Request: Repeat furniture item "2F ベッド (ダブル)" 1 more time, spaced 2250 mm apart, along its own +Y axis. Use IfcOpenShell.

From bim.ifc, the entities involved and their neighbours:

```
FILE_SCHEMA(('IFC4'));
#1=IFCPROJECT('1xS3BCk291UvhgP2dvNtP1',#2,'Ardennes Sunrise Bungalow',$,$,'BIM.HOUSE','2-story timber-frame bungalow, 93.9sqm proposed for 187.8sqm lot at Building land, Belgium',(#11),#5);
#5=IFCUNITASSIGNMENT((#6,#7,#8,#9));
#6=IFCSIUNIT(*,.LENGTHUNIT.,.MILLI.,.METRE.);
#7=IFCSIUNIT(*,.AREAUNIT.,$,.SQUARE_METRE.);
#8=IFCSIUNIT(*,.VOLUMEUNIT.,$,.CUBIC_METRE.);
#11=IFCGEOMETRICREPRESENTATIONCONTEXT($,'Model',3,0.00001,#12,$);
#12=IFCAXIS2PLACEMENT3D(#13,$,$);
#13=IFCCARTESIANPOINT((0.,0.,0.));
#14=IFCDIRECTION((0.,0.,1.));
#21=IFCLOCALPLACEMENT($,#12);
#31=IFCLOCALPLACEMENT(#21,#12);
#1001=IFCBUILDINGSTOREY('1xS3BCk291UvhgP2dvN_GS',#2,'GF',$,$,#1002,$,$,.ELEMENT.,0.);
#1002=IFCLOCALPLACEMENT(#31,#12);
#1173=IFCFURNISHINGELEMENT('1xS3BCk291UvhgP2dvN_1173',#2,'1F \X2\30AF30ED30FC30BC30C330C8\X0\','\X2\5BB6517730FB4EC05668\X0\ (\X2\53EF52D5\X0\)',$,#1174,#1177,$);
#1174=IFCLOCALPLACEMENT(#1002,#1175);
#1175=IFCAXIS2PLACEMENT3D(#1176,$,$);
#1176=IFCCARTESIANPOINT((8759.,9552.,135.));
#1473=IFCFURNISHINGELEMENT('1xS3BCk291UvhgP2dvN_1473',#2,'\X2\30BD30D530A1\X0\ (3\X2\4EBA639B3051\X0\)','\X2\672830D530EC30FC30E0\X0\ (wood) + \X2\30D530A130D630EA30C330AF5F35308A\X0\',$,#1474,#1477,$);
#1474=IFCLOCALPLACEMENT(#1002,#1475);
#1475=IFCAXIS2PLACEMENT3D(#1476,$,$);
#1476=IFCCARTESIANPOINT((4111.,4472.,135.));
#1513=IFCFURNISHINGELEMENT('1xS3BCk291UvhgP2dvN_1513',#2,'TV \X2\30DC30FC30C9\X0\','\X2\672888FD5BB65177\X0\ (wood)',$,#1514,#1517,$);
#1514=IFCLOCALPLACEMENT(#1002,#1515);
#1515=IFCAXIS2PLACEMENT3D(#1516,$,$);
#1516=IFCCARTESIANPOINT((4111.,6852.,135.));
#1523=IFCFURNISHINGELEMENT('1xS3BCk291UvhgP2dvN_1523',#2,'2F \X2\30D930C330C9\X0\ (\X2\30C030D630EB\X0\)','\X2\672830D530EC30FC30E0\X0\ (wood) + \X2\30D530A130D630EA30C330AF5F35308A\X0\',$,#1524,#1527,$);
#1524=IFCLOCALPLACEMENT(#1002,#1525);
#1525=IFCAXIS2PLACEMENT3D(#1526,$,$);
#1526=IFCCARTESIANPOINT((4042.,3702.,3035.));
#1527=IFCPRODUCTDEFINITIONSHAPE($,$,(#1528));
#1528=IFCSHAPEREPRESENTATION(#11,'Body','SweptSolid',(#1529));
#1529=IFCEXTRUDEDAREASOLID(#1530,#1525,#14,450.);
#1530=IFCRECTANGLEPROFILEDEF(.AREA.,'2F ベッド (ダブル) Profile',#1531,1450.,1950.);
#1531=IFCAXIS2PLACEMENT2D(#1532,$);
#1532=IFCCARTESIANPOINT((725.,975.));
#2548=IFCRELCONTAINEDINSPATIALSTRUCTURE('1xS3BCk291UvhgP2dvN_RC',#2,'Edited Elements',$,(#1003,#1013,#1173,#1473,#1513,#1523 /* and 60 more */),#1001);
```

```python
import ifcopenshell
import ifcopenshell.api.geometry
import ifcopenshell.api.root
import ifcopenshell.util.element
import ifcopenshell.util.placement

model = ifcopenshell.open("bim.ifc")


def reuse_history(source, copy):
    """copy_class also copies each property set's owner history, people and application; keep the originals."""
    for rel in copy.IsDefinedBy:
        if rel.is_a("IfcRelDefinesByProperties") and (history := rel.RelatingPropertyDefinition.OwnerHistory):
            rel.RelatingPropertyDefinition.OwnerHistory = source.OwnerHistory
            ifcopenshell.util.element.remove_deep2(model, history)


source = model.by_guid("1xS3BCk291UvhgP2dvN_1523")
base = ifcopenshell.util.placement.get_local_placement(source.ObjectPlacement)
step = base[:3, 1] * 2250.0

for i in range(1, 2):
    copy = ifcopenshell.api.root.copy_class(model, product=source)
    copy.Representation = ifcopenshell.util.element.copy_deep(
        model, source.Representation, exclude=["IfcGeometricRepresentationContext", "IfcRepresentationMap"]
    )
    reuse_history(source, copy)
    matrix = base.copy()
    matrix[:3, 3] += i * step
    print("added at", matrix[:3, 3].round(3) + 0.0)
    ifcopenshell.api.geometry.edit_object_placement(model, product=copy, matrix=matrix, is_si=False)

model.write("bim_v2.ifc")
```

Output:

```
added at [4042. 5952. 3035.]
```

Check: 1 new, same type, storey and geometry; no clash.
